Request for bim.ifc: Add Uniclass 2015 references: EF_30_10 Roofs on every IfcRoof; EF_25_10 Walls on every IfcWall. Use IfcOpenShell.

First a look at what the model holds.

```python
import ifcopenshell

model = ifcopenshell.open("bim.ifc")
print(model.schema)
print("classifications:", [c.Name for c in model.by_type("IfcClassification")])
for ifc_class in ("IfcDoor", "IfcRoof", "IfcStair", "IfcWall", "IfcWindow"):
    print(ifc_class, len(model.by_type(ifc_class)))
```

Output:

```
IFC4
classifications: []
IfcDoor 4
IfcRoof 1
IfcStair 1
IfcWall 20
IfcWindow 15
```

```python
import ifcopenshell
import ifcopenshell.api.classification

model = ifcopenshell.open("bim.ifc")

system = ifcopenshell.api.classification.add_classification(model, classification="Uniclass 2015")

codes = {
    "IfcRoof": ("EF_30_10", "Roofs"),
    "IfcWall": ("EF_25_10", "Walls"),
}
for ifc_class, (code, name) in codes.items():
    products = model.by_type(ifc_class)
    ifcopenshell.api.classification.add_reference(
        model, products=products, classification=system, identification=code, name=name
    )
    print(code, len(products))

model.write("bim-out.ifc")
```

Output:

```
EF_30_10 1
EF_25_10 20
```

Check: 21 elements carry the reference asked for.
